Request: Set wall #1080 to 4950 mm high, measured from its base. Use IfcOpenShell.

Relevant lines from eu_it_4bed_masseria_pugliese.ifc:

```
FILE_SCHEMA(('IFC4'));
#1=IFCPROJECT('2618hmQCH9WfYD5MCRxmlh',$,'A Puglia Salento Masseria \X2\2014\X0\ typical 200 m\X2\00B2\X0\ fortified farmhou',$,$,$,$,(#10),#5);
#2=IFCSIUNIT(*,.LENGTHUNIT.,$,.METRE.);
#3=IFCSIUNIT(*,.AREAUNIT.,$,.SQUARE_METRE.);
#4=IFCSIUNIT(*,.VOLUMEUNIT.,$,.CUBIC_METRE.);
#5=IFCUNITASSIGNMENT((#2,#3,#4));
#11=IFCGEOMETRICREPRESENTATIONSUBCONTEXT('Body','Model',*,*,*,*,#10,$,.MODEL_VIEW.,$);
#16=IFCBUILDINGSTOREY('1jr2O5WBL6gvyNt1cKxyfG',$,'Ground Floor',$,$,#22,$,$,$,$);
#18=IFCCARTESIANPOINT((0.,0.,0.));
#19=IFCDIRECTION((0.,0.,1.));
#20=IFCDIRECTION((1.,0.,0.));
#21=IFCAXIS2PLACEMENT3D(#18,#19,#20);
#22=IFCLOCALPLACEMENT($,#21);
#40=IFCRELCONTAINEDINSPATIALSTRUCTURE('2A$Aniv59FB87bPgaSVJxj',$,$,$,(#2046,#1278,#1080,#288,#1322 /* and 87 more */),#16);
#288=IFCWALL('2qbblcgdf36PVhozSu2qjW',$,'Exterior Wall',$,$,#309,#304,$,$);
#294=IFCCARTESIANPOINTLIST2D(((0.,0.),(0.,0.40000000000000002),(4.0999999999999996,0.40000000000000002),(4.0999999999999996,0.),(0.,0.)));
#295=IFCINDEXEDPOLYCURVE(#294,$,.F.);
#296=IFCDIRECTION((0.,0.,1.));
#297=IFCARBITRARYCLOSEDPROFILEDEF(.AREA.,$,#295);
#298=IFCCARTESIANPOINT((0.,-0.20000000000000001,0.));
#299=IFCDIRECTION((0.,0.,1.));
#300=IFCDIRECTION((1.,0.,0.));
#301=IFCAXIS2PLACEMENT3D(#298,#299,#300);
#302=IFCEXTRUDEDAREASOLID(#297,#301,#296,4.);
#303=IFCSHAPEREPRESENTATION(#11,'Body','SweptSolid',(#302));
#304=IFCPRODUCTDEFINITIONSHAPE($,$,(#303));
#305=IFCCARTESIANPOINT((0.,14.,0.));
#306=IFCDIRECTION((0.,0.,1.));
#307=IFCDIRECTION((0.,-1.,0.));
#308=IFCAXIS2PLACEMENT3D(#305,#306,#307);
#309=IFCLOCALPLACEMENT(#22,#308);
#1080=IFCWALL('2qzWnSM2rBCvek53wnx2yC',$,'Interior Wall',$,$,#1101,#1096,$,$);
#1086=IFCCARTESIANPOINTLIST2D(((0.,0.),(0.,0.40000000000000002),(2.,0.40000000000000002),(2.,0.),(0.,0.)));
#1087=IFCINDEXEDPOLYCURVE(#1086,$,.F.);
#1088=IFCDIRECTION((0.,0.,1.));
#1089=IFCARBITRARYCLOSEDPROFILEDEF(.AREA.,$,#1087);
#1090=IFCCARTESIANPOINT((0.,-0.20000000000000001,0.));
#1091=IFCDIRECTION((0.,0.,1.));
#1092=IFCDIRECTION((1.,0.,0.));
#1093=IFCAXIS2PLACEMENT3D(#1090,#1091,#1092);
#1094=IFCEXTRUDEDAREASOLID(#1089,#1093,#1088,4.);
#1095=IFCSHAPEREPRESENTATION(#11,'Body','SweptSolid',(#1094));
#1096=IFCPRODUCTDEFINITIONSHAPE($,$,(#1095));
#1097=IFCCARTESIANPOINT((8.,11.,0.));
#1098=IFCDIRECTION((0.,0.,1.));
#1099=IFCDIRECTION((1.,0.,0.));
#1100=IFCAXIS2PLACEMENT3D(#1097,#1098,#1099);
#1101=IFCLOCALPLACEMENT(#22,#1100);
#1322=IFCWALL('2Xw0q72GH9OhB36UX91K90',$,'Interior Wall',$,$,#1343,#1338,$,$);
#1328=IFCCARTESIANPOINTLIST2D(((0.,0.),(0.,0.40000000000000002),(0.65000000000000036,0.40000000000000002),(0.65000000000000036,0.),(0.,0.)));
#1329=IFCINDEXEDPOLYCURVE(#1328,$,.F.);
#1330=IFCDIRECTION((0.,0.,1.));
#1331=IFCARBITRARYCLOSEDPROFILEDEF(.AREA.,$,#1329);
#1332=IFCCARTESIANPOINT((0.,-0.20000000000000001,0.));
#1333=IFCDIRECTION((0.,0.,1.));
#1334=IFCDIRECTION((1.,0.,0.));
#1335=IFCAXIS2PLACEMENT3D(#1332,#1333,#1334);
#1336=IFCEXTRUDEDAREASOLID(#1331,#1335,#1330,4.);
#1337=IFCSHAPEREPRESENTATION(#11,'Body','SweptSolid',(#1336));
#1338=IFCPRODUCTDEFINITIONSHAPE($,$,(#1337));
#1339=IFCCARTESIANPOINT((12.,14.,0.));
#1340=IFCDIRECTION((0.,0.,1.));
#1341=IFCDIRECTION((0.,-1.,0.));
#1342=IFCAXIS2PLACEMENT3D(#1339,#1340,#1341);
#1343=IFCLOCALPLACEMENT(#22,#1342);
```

```python
import ifcopenshell
import ifcopenshell.geom
import ifcopenshell.util.representation
import ifcopenshell.util.shape
import ifcopenshell.util.unit

model = ifcopenshell.open("eu_it_4bed_masseria_pugliese.ifc")
unit_scale = ifcopenshell.util.unit.calculate_unit_scale(model)
settings = ifcopenshell.geom.settings()


def volume(element):
    """Net volume in cubic metres, openings subtracted."""
    shape = ifcopenshell.geom.create_shape(settings, element)
    return ifcopenshell.util.shape.get_volume(shape.geometry)


wall = model.by_guid("2qzWnSM2rBCvek53wnx2yC")
before = volume(wall)

body = ifcopenshell.util.representation.get_representation(wall, "Model", "Body")
solid = body.Items[0]
old_height = solid.Depth
solid.Depth = 4.95 / unit_scale
after = volume(wall)

print(f"height {old_height:g} -> {solid.Depth:g}, volume {before:.3f} -> {after:.3f} m3")

model.write("eu_it_4bed_masseria_pugliese_rev.ifc")
```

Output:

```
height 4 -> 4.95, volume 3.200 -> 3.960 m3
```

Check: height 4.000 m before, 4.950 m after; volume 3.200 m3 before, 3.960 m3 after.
